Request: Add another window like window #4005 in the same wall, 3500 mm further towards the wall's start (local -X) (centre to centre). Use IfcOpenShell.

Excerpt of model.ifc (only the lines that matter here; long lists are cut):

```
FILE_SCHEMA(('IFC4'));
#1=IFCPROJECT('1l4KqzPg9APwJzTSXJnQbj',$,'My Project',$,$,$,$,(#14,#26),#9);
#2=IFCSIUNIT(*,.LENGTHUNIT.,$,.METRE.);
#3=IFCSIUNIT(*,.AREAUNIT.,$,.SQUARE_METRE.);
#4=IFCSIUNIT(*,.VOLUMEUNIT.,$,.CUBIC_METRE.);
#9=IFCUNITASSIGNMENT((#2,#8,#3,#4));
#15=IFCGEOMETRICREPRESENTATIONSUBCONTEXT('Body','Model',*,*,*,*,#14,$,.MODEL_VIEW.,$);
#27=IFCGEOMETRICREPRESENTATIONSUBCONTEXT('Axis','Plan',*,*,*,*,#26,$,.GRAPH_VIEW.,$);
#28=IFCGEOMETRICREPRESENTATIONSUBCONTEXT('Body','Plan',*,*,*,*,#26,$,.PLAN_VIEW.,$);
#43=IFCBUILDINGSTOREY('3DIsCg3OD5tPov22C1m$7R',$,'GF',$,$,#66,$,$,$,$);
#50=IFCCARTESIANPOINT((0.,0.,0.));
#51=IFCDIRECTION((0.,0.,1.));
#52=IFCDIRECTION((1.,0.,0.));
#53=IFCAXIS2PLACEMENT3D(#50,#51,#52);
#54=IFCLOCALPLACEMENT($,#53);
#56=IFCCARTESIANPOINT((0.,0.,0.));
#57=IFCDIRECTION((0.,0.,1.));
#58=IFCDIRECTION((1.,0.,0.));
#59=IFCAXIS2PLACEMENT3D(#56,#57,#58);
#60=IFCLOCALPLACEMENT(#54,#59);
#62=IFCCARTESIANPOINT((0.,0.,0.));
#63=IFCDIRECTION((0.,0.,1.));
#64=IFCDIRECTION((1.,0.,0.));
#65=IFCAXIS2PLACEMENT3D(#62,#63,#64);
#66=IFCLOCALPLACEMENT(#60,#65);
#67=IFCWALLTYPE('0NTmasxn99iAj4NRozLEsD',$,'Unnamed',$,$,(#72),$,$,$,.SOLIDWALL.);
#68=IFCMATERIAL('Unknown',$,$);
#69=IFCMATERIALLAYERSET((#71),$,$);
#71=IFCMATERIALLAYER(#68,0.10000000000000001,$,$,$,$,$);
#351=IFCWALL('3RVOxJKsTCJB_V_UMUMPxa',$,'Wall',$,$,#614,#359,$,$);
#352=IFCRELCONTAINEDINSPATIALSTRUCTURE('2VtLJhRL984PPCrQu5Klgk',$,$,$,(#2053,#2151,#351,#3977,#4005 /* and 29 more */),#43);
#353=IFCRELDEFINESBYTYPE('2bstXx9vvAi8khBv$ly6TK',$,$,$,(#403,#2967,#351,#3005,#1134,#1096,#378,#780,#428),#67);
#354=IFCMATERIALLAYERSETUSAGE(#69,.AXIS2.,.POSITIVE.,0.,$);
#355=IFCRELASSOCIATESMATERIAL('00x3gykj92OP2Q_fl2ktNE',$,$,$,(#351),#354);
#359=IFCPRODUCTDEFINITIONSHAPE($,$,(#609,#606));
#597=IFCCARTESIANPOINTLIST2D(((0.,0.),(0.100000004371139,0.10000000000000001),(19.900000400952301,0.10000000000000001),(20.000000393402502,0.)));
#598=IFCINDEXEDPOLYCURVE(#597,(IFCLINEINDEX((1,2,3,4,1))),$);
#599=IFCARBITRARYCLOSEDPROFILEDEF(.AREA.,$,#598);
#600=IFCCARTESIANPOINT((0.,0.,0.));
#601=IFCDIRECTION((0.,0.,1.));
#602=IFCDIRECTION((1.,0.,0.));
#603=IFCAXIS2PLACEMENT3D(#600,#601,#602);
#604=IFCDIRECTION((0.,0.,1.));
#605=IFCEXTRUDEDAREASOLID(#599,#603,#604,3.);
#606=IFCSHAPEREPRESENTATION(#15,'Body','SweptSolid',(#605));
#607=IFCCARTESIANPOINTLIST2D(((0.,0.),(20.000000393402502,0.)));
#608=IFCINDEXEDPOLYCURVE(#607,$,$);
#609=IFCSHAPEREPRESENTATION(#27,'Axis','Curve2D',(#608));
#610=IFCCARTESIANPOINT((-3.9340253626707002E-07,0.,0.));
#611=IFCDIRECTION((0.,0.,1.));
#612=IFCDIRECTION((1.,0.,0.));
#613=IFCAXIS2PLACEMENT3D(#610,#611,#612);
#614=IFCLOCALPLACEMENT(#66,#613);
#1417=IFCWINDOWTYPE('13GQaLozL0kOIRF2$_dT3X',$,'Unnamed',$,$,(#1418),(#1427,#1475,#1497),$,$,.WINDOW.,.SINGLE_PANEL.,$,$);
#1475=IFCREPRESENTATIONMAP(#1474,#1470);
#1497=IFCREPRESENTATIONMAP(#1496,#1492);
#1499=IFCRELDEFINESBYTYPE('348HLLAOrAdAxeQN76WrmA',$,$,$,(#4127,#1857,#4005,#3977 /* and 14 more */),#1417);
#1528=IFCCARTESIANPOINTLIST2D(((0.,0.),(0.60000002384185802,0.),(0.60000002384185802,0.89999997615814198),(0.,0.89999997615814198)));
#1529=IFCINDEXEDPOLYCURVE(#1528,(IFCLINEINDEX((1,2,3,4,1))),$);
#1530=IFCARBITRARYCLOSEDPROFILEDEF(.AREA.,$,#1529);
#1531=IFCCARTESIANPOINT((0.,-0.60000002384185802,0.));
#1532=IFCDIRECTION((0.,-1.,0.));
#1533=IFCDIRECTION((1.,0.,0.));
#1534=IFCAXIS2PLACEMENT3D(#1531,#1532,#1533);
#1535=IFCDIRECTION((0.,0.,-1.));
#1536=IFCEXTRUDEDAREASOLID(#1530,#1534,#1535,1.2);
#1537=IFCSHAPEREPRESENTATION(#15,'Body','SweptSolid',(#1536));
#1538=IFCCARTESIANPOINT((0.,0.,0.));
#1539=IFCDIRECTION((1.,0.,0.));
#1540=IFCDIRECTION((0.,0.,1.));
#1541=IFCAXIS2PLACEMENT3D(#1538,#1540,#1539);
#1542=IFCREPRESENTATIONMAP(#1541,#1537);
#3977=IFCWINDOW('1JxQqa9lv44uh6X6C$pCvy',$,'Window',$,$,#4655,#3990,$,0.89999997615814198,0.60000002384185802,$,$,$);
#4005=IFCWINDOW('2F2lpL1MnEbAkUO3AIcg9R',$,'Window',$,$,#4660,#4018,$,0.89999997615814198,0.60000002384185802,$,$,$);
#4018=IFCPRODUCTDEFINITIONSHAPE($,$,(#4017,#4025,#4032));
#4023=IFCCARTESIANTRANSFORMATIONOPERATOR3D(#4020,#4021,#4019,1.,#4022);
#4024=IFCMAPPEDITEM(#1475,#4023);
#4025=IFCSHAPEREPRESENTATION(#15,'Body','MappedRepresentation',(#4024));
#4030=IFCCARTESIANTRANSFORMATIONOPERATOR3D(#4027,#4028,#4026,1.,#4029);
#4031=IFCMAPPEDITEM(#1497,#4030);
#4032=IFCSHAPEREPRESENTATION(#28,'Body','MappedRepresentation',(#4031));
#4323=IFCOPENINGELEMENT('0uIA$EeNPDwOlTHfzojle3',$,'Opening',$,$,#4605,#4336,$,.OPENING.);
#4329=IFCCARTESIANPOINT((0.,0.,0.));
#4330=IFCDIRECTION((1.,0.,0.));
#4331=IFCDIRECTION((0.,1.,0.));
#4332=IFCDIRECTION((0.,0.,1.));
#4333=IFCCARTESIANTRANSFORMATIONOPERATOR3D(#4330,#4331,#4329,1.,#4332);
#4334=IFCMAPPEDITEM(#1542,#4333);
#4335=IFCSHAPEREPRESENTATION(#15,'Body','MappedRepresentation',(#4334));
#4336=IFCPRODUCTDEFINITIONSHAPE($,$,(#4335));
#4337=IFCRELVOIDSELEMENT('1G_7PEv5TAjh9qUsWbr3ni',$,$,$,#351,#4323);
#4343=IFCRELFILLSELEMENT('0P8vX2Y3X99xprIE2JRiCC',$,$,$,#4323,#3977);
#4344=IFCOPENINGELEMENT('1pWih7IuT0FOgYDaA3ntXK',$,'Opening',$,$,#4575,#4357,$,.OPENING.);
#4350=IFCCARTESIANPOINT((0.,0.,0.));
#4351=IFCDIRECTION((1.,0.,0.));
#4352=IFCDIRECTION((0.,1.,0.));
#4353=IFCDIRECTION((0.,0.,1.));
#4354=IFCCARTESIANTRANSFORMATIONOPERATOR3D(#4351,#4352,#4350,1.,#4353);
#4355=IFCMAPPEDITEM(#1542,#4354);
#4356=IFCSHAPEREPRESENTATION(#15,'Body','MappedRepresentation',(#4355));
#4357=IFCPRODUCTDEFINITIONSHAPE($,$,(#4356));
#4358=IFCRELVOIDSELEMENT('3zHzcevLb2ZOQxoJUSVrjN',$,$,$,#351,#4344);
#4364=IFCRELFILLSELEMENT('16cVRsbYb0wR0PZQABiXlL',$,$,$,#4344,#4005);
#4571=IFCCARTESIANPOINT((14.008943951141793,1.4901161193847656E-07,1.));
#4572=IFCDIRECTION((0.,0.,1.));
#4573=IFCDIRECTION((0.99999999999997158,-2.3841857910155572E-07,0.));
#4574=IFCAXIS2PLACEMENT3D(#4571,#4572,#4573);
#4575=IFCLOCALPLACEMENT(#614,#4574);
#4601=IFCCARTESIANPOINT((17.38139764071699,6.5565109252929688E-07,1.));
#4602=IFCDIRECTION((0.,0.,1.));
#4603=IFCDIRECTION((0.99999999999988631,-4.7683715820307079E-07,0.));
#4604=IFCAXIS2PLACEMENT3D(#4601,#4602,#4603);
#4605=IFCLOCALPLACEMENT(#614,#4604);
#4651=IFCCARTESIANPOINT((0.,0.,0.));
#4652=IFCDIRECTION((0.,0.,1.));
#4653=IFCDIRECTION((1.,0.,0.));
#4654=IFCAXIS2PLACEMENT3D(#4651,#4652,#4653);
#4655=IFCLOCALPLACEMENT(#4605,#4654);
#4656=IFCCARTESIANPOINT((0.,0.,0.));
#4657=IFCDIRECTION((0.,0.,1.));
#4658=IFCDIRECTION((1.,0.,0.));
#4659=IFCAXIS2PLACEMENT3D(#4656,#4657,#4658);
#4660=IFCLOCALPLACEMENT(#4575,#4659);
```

```python
import ifcopenshell
import ifcopenshell.api.feature
import ifcopenshell.api.geometry
import ifcopenshell.api.root
import ifcopenshell.geom
import ifcopenshell.util.element
import ifcopenshell.util.placement
import ifcopenshell.util.shape

model = ifcopenshell.open("model.ifc")
settings = ifcopenshell.geom.settings()


def volume(element):
    """Net volume in cubic metres, openings subtracted."""
    shape = ifcopenshell.geom.create_shape(settings, element)
    return ifcopenshell.util.shape.get_volume(shape.geometry)


window = model.by_id(4005)
opening = window.FillsVoids[0].RelatingOpeningElement
wall = opening.VoidsElements[0].RelatingBuildingElement
before = volume(wall)
shift = ifcopenshell.util.placement.get_local_placement(wall.ObjectPlacement)[:3, 0] * -3.5

# copy_class copies the void relationship, type, container and properties, but no geometry.
new_opening = ifcopenshell.api.root.copy_class(model, product=opening)
new_opening.Representation = ifcopenshell.util.element.copy_deep(
    model, opening.Representation, exclude=["IfcGeometricRepresentationContext", "IfcRepresentationMap"]
)
new_window = ifcopenshell.api.root.copy_class(model, product=window)
new_window.Representation = ifcopenshell.util.element.copy_deep(
    model, window.Representation, exclude=["IfcGeometricRepresentationContext", "IfcRepresentationMap"]
)
ifcopenshell.api.feature.add_filling(model, opening=new_opening, element=new_window)

for old, new in ((opening, new_opening), (window, new_window)):
    matrix = ifcopenshell.util.placement.get_local_placement(old.ObjectPlacement)
    matrix[:3, 3] += shift
    ifcopenshell.api.geometry.edit_object_placement(model, product=new, matrix=matrix, is_si=False)

after = volume(wall)

print(f"wall volume {before:.3f} -> {after:.3f} m3")

model.write("model_edited.ifc")
```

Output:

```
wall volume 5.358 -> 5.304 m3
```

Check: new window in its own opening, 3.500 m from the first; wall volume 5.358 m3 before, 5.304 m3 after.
